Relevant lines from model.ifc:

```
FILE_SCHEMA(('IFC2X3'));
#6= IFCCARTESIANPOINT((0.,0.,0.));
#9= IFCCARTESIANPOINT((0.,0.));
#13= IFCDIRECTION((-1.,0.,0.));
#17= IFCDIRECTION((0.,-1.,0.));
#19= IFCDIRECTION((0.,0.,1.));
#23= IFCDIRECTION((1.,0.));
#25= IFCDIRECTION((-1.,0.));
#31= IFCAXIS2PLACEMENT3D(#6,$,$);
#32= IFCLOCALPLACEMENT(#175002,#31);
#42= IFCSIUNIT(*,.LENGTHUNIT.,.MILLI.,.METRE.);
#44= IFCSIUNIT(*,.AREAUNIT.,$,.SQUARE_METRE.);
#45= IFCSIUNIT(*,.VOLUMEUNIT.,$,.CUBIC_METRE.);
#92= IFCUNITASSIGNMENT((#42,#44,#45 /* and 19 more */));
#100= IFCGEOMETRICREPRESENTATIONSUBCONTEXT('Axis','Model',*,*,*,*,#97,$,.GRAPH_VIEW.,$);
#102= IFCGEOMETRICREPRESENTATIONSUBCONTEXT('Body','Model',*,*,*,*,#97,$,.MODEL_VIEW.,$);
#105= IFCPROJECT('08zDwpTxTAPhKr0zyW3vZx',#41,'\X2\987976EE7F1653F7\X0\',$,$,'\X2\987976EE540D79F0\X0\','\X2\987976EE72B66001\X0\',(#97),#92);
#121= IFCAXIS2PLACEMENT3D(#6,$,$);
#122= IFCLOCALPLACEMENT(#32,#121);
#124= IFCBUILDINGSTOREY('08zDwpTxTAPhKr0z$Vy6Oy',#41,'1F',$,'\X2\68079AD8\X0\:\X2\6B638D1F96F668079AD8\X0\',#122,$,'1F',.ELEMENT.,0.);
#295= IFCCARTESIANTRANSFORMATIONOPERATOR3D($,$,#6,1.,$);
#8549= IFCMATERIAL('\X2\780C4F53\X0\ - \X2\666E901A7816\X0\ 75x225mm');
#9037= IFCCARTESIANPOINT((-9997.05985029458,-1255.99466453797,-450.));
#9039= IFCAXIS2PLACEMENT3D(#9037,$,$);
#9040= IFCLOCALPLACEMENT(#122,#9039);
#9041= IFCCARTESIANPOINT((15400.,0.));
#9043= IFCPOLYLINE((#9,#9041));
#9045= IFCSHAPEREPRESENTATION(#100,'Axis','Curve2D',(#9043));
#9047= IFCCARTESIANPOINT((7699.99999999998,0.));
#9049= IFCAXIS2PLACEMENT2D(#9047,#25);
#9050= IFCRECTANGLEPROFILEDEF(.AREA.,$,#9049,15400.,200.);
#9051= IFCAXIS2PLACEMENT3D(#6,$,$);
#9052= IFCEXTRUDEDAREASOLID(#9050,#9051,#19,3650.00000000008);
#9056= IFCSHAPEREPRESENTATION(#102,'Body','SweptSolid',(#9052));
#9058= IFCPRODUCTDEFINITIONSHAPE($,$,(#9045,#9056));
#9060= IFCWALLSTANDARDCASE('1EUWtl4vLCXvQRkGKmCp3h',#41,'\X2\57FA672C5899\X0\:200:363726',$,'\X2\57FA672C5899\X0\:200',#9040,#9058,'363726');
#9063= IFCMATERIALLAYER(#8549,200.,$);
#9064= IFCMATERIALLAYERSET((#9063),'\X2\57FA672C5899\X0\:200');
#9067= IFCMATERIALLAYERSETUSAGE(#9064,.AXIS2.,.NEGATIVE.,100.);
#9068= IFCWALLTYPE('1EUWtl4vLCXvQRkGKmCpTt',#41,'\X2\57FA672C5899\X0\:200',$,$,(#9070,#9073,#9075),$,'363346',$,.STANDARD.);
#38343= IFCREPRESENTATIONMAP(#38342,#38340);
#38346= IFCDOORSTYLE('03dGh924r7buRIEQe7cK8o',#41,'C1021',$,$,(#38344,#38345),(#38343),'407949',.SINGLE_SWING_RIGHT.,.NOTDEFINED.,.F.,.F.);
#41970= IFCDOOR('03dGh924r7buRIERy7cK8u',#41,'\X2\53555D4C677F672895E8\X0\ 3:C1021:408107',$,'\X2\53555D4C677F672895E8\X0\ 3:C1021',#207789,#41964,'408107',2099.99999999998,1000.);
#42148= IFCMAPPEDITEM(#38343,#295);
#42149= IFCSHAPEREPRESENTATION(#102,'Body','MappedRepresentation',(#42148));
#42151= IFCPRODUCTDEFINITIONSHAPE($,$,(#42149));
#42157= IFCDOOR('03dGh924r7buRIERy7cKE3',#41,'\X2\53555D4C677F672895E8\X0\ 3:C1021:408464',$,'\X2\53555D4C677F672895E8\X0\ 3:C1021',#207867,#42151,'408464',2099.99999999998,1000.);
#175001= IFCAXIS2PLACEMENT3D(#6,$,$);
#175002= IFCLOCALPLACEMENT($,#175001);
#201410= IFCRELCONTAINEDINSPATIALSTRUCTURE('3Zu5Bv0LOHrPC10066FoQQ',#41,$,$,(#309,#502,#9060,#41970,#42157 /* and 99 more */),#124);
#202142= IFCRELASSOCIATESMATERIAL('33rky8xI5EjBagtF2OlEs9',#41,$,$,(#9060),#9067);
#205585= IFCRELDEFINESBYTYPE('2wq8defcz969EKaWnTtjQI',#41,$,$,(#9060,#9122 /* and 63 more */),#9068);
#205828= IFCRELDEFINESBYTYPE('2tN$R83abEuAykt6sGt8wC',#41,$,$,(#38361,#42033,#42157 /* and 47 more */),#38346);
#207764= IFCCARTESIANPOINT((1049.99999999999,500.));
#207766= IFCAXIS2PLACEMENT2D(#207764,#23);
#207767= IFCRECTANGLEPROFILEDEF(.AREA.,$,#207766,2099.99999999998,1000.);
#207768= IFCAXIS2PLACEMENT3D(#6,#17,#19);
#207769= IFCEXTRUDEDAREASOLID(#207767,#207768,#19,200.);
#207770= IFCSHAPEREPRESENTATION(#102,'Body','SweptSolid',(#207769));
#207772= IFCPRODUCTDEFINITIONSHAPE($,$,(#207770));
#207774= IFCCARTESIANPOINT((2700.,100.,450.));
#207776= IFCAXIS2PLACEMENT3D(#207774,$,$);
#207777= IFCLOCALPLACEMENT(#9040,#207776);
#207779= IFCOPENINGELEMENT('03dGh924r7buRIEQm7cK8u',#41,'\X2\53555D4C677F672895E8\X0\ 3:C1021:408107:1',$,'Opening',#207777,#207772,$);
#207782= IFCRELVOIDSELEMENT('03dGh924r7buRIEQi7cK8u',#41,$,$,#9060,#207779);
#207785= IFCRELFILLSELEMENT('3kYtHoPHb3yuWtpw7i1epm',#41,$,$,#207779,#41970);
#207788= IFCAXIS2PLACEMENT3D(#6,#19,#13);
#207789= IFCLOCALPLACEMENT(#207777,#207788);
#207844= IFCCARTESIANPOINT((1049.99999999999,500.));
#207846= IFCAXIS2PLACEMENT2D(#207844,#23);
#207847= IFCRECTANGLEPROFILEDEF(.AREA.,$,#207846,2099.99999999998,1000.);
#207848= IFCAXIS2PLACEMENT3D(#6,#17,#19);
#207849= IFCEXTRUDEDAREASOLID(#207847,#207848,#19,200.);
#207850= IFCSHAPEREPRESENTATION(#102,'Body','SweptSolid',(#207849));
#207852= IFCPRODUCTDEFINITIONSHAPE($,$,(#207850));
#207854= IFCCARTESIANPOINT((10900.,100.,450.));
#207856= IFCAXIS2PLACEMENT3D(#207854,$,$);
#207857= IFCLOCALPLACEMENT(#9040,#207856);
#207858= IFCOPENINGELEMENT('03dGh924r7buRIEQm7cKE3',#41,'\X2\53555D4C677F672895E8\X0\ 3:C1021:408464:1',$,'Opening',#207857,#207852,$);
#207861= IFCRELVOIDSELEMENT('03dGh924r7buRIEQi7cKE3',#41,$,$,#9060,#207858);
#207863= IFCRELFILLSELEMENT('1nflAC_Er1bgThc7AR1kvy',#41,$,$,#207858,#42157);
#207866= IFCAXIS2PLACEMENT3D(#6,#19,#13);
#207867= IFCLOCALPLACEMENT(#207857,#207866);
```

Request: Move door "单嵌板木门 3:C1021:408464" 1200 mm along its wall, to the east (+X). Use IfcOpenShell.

```python
import ifcopenshell
import ifcopenshell.api.geometry
import ifcopenshell.util.placement
import ifcopenshell.util.unit

model = ifcopenshell.open("model.ifc")
unit_scale = ifcopenshell.util.unit.calculate_unit_scale(model)

door = model.by_guid("03dGh924r7buRIERy7cKE3")
opening = door.FillsVoids[0].RelatingOpeningElement
wall = opening.VoidsElements[0].RelatingBuildingElement

wall_matrix = ifcopenshell.util.placement.get_local_placement(wall.ObjectPlacement)
shift = wall_matrix[:3, 0] * 1.2 / unit_scale
before = ifcopenshell.util.placement.get_local_placement(door.ObjectPlacement)[:3, 3].copy()

# The door is placed relative to its opening, so it follows when the opening moves.
matrix = ifcopenshell.util.placement.get_local_placement(opening.ObjectPlacement)
matrix[:3, 3] += shift
ifcopenshell.api.geometry.edit_object_placement(
    model, product=opening, matrix=matrix, is_si=False, should_transform_children=True
)

after = ifcopenshell.util.placement.get_local_placement(door.ObjectPlacement)[:3, 3]
print("door moved by", (after - before).round(3) + 0.0)

model.write("model_updated.ifc")
```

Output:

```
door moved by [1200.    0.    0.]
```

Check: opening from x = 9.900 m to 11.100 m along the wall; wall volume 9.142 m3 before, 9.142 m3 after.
